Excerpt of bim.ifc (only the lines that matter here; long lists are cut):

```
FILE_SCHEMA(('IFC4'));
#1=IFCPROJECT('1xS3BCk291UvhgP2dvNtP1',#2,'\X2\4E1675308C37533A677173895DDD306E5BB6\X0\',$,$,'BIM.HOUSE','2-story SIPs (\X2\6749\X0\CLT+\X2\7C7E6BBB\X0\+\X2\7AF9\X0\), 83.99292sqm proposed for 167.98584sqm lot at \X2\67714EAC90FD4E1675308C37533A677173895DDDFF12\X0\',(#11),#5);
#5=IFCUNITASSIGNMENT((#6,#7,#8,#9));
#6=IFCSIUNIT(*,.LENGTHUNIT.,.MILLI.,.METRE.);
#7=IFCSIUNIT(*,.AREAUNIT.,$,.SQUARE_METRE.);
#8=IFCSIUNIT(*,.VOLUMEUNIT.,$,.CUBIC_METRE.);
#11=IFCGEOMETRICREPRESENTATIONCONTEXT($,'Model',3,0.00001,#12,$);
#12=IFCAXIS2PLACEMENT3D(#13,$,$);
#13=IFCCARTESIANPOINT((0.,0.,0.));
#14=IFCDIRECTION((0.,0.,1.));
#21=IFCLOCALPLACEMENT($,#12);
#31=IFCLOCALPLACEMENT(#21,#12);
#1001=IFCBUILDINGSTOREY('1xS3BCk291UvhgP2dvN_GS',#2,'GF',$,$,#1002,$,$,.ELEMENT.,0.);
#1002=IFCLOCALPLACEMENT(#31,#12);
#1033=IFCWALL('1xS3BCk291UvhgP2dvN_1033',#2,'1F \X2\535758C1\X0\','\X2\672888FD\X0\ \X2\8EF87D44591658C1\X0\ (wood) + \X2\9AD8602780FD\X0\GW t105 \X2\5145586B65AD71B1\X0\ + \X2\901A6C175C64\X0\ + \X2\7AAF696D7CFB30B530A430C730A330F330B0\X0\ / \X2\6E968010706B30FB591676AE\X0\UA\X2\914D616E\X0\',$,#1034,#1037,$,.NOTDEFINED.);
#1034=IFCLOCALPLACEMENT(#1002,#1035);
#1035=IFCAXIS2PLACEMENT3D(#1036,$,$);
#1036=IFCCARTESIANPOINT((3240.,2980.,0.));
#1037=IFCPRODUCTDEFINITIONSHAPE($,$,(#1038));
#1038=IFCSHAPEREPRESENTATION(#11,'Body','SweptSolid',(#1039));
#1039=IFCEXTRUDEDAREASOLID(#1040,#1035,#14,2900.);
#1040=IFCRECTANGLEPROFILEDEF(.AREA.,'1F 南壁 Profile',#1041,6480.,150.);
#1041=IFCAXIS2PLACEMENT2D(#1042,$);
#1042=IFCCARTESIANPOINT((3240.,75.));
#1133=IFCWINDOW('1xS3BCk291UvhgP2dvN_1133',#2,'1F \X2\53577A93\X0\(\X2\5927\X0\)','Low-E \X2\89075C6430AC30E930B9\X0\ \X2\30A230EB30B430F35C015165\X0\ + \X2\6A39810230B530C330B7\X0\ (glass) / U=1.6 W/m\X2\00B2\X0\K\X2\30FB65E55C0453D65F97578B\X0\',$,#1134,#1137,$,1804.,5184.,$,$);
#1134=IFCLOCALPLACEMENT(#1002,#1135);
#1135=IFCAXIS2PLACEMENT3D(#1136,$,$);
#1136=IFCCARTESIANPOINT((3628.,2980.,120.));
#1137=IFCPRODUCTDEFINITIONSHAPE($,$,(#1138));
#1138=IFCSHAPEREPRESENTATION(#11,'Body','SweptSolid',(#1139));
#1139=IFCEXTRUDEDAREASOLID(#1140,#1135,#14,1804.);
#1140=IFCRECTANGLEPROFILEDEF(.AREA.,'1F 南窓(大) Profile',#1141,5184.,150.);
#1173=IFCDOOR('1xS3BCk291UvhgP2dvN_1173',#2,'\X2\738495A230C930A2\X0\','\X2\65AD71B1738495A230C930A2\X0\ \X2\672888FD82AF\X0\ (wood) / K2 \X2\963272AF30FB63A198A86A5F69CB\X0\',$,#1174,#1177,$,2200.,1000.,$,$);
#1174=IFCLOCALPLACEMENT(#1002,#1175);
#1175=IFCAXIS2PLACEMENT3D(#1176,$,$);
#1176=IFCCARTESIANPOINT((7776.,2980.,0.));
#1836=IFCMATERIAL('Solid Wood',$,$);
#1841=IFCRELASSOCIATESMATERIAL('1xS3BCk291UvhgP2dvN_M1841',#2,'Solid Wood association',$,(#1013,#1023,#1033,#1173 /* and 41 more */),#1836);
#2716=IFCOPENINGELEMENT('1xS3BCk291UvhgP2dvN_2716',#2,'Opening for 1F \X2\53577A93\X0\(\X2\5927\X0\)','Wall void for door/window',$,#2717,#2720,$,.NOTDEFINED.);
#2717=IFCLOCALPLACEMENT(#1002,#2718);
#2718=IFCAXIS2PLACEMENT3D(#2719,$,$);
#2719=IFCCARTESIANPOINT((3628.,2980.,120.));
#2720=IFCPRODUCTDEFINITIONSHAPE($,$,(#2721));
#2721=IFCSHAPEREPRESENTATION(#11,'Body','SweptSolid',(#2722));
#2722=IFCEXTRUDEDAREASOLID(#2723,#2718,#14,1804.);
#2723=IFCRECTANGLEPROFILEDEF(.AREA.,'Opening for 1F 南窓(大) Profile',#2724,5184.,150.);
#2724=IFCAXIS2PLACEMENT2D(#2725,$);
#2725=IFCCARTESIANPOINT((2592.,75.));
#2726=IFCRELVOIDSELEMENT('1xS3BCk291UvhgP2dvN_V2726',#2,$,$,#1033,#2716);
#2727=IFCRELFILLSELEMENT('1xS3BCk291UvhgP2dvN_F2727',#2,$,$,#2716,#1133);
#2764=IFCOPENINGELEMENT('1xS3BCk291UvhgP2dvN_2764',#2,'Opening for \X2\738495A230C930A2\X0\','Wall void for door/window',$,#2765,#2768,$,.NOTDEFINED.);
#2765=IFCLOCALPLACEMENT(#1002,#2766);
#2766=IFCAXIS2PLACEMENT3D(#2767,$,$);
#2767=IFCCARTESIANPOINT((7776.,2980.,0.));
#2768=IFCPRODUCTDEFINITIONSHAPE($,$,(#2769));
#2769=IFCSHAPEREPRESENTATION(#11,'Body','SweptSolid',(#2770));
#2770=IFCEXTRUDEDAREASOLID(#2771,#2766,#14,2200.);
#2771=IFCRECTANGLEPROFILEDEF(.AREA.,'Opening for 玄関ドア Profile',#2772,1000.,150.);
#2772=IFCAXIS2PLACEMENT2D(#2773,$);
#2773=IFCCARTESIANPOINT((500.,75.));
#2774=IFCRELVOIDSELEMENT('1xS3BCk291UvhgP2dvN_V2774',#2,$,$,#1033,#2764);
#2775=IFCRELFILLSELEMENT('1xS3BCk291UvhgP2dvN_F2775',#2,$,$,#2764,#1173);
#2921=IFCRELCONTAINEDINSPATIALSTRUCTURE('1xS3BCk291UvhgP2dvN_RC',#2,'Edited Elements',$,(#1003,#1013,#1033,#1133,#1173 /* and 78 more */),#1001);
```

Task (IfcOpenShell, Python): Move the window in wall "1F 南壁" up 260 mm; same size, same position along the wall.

```python
import numpy as np
import ifcopenshell
import ifcopenshell.api.geometry
import ifcopenshell.util.placement
import ifcopenshell.util.unit

model = ifcopenshell.open("bim.ifc")
unit_scale = ifcopenshell.util.unit.calculate_unit_scale(model)

window = model.by_guid("1xS3BCk291UvhgP2dvN_1133")
opening = window.FillsVoids[0].RelatingOpeningElement
dz = 260.0

shift = np.array([0.0, 0.0, dz])
# The window is not placed relative to its opening, so move both.
for product in (opening, window):
    matrix = ifcopenshell.util.placement.get_local_placement(product.ObjectPlacement)
    matrix[:3, 3] += shift
    ifcopenshell.api.geometry.edit_object_placement(model, product=product, matrix=matrix, is_si=False)

print(f"moved by {dz * unit_scale:+.3f} m")

model.write("bim_edited.ifc")
```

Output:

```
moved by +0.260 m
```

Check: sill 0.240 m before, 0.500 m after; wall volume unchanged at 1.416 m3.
